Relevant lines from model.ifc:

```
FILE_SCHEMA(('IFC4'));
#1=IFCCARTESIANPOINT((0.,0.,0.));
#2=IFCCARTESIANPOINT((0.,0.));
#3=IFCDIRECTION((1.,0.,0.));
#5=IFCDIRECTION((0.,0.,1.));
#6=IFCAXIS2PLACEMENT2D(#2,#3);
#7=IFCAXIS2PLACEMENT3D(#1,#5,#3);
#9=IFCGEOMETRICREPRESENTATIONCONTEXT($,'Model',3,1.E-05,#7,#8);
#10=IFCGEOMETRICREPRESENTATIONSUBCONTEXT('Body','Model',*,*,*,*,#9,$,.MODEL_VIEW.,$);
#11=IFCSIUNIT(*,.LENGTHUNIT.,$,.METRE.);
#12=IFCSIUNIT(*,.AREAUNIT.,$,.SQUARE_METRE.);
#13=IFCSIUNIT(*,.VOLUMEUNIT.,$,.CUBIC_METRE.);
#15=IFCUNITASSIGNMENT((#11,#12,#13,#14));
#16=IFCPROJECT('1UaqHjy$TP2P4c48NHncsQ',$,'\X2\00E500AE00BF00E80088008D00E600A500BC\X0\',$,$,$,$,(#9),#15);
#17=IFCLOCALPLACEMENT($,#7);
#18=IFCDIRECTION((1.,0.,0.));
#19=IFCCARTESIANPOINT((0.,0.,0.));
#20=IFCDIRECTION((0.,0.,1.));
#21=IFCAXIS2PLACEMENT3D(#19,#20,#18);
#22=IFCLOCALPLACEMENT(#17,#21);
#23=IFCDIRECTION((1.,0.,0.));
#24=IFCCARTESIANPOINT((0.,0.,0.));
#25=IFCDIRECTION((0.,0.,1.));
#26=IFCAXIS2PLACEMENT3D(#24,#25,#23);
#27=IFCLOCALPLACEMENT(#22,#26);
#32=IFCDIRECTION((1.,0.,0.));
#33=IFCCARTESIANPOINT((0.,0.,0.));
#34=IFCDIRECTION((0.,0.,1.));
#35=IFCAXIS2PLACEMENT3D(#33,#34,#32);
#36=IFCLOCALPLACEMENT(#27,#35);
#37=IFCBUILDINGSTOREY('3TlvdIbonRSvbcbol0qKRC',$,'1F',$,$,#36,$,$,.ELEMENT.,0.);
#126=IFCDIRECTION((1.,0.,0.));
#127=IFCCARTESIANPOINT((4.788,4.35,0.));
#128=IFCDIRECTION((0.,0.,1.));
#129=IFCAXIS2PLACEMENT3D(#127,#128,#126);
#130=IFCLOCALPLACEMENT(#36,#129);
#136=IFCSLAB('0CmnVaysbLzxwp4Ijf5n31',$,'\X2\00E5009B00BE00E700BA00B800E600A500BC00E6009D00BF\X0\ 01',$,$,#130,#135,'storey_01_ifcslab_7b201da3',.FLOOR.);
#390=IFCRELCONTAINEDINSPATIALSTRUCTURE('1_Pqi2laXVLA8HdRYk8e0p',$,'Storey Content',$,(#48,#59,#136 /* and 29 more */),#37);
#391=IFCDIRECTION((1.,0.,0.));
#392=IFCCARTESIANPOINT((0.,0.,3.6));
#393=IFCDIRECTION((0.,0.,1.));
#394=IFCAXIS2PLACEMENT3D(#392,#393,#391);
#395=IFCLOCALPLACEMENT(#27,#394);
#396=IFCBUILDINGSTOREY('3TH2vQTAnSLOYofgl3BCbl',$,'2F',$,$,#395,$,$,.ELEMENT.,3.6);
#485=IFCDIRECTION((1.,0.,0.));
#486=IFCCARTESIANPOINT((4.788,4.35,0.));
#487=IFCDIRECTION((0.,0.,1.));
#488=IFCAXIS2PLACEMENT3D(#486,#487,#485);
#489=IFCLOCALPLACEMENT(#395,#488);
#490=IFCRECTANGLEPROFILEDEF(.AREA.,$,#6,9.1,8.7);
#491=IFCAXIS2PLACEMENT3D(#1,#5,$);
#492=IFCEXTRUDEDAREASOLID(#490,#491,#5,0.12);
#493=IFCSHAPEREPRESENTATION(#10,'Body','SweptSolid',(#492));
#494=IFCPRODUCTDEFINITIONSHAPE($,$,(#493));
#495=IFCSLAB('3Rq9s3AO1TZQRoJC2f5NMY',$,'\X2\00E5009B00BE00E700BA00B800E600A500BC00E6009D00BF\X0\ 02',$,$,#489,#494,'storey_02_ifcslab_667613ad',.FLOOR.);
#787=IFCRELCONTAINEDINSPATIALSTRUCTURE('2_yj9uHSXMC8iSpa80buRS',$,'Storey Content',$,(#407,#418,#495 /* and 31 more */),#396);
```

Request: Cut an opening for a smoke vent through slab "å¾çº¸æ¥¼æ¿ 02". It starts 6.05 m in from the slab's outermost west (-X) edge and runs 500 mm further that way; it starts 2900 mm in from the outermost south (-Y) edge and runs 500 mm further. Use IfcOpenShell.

```python
import numpy as np
import ifcopenshell
import ifcopenshell.api.feature
import ifcopenshell.api.geometry
import ifcopenshell.api.root
import ifcopenshell.geom
import ifcopenshell.util.placement
import ifcopenshell.util.representation
import ifcopenshell.util.shape
import ifcopenshell.util.unit

model = ifcopenshell.open("model.ifc")
unit_scale = ifcopenshell.util.unit.calculate_unit_scale(model)
settings = ifcopenshell.geom.settings()


def volume(element):
    """Net volume in cubic metres, openings subtracted."""
    shape = ifcopenshell.geom.create_shape(settings, element)
    return ifcopenshell.util.shape.get_volume(shape.geometry)


slab = model.by_guid("3Rq9s3AO1TZQRoJC2f5NMY")
before = volume(slab)

# Extent in the slab's own axes, in metres. The edges named are its -X and -Y sides.
slab_shape = ifcopenshell.geom.create_shape(settings, slab)
vertices = ifcopenshell.util.shape.get_vertices(slab_shape.geometry)
x_min, y_min, bottom = vertices.min(axis=0)
top = vertices[:, 2].max()

opening = ifcopenshell.api.root.create_entity(model, ifc_class="IfcOpeningElement", name="Smoke vent opening", predefined_type="OPENING")
context = ifcopenshell.util.representation.get_context(model, "Model", "Body", "MODEL_VIEW")
width, depth = 0.5, 0.5
outline = [(0.0, 0.0), (width, 0.0), (width, depth), (0.0, depth), (0.0, 0.0)]
# Overshoot both faces by 50 mm so the cut is clean.
shape = ifcopenshell.api.geometry.add_slab_representation(
    model, context=context, depth=top - bottom + 0.1, polyline=outline
)
ifcopenshell.api.geometry.assign_representation(model, product=opening, representation=shape)

matrix = ifcopenshell.util.placement.get_local_placement(slab.ObjectPlacement)
matrix[:, 3] = matrix @ np.append(np.array([x_min + 6.05, y_min + 2.9, bottom - 0.05]) / unit_scale, 1.0)
ifcopenshell.api.geometry.edit_object_placement(model, product=opening, matrix=matrix, is_si=False)
ifcopenshell.api.feature.add_feature(model, feature=opening, element=slab)

after = volume(slab)

print(f"slab volume {before:.3f} -> {after:.3f} m3")

model.write("model_v2.ifc")
```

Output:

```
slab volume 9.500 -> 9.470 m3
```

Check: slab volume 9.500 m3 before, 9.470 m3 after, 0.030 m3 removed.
